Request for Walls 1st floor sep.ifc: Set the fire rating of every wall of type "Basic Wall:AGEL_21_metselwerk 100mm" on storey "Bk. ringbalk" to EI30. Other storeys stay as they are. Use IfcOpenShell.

First a look at what the model holds.

```python
import ifcopenshell
import ifcopenshell.util.element

model = ifcopenshell.open("Walls 1st floor sep.ifc")
print(model.schema)
storey = next(s for s in model.by_type("IfcBuildingStorey") if s.Name == "Bk. ringbalk")
walls = [e for e in ifcopenshell.util.element.get_decomposition(storey) if e.is_a("IfcWall")]
seen = {}
for e in walls:
    element_type = ifcopenshell.util.element.get_type(e)
    key = (element_type.Name if element_type != e and element_type else None, ifcopenshell.util.element.get_pset(e, "Pset_WallCommon", "FireRating"))
    seen[key] = seen.get(key, 0) + 1
for (name, value), count in sorted(seen.items(), key=str):
    print(count, "x", name, "|", value)
```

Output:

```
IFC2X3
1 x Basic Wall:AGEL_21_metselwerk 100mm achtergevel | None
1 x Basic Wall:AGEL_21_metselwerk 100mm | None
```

```python
import ifcopenshell
import ifcopenshell.api.pset
import ifcopenshell.util.element

model = ifcopenshell.open("Walls 1st floor sep.ifc")

storey = next(s for s in model.by_type("IfcBuildingStorey") if s.Name == "Bk. ringbalk")
walls = [e for e in ifcopenshell.util.element.get_decomposition(storey) if e.is_a("IfcWall")]

count = 0
for e in walls:
    element_type = ifcopenshell.util.element.get_type(e)
    if element_type in (None, e) or element_type.Name != "Basic Wall:AGEL_21_metselwerk 100mm":
        continue
    # add_pset returns the element's existing set when there is one.
    pset = ifcopenshell.api.pset.add_pset(model, product=e, name="Pset_WallCommon")
    ifcopenshell.api.pset.edit_pset(model, pset=pset, properties={"FireRating": "EI30"})
    count += 1

print(count, "walls updated")

model.write("Walls 1st floor sep-out.ifc")
```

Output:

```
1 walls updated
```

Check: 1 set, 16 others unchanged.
